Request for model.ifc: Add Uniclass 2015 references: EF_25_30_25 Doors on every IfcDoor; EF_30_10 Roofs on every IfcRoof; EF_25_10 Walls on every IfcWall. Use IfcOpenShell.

First a look at what the model holds.

```python
import ifcopenshell

model = ifcopenshell.open("model.ifc")
print(model.schema)
print("classifications:", [c.Name for c in model.by_type("IfcClassification")])
for ifc_class in ("IfcDoor", "IfcRoof", "IfcStair", "IfcWall", "IfcWindow"):
    print(ifc_class, len(model.by_type(ifc_class)))
```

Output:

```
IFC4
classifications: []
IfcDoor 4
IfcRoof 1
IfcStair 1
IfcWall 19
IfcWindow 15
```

```python
import ifcopenshell
import ifcopenshell.api.classification

model = ifcopenshell.open("model.ifc")

system = ifcopenshell.api.classification.add_classification(model, classification="Uniclass 2015")

codes = {
    "IfcDoor": ("EF_25_30_25", "Doors"),
    "IfcRoof": ("EF_30_10", "Roofs"),
    "IfcWall": ("EF_25_10", "Walls"),
}
for ifc_class, (code, name) in codes.items():
    products = model.by_type(ifc_class)
    ifcopenshell.api.classification.add_reference(
        model, products=products, classification=system, identification=code, name=name
    )
    print(code, len(products))

model.write("model_updated.ifc")
```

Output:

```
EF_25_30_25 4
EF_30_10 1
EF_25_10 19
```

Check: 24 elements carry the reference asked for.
